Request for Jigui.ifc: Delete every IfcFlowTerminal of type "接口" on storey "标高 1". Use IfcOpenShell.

First a look at what the model holds.

```python
import ifcopenshell
import ifcopenshell.util.element

model = ifcopenshell.open("Jigui.ifc")
print(model.schema)
storey = next(s for s in model.by_type("IfcBuildingStorey") if s.Name == "标高 1")
terminals = [e for e in ifcopenshell.util.element.get_decomposition(storey) if e.is_a("IfcFlowTerminal")]
seen = {}
for e in terminals:
    element_type = ifcopenshell.util.element.get_type(e)
    name = element_type.Name if element_type not in (None, e) else None
    seen[name] = seen.get(name, 0) + 1
for name, count in sorted(seen.items(), key=str):
    print(count, "x", name)
```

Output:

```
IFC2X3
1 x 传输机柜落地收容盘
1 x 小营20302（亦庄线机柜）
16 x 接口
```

```python
import ifcopenshell
import ifcopenshell.api.root
import ifcopenshell.util.element

model = ifcopenshell.open("Jigui.ifc")

storey = next(s for s in model.by_type("IfcBuildingStorey") if s.Name == "标高 1")
terminals = [e for e in ifcopenshell.util.element.get_decomposition(storey) if e.is_a("IfcFlowTerminal")]
targets = [e for e in terminals if (t := ifcopenshell.util.element.get_type(e)) not in (None, e) and t.Name == "接口"]

for e in targets:
    ifcopenshell.api.root.remove_product(model, product=e)
print(len(targets), "removed")

model.write("Jigui_rev.ifc")
```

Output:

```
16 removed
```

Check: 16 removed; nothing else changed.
